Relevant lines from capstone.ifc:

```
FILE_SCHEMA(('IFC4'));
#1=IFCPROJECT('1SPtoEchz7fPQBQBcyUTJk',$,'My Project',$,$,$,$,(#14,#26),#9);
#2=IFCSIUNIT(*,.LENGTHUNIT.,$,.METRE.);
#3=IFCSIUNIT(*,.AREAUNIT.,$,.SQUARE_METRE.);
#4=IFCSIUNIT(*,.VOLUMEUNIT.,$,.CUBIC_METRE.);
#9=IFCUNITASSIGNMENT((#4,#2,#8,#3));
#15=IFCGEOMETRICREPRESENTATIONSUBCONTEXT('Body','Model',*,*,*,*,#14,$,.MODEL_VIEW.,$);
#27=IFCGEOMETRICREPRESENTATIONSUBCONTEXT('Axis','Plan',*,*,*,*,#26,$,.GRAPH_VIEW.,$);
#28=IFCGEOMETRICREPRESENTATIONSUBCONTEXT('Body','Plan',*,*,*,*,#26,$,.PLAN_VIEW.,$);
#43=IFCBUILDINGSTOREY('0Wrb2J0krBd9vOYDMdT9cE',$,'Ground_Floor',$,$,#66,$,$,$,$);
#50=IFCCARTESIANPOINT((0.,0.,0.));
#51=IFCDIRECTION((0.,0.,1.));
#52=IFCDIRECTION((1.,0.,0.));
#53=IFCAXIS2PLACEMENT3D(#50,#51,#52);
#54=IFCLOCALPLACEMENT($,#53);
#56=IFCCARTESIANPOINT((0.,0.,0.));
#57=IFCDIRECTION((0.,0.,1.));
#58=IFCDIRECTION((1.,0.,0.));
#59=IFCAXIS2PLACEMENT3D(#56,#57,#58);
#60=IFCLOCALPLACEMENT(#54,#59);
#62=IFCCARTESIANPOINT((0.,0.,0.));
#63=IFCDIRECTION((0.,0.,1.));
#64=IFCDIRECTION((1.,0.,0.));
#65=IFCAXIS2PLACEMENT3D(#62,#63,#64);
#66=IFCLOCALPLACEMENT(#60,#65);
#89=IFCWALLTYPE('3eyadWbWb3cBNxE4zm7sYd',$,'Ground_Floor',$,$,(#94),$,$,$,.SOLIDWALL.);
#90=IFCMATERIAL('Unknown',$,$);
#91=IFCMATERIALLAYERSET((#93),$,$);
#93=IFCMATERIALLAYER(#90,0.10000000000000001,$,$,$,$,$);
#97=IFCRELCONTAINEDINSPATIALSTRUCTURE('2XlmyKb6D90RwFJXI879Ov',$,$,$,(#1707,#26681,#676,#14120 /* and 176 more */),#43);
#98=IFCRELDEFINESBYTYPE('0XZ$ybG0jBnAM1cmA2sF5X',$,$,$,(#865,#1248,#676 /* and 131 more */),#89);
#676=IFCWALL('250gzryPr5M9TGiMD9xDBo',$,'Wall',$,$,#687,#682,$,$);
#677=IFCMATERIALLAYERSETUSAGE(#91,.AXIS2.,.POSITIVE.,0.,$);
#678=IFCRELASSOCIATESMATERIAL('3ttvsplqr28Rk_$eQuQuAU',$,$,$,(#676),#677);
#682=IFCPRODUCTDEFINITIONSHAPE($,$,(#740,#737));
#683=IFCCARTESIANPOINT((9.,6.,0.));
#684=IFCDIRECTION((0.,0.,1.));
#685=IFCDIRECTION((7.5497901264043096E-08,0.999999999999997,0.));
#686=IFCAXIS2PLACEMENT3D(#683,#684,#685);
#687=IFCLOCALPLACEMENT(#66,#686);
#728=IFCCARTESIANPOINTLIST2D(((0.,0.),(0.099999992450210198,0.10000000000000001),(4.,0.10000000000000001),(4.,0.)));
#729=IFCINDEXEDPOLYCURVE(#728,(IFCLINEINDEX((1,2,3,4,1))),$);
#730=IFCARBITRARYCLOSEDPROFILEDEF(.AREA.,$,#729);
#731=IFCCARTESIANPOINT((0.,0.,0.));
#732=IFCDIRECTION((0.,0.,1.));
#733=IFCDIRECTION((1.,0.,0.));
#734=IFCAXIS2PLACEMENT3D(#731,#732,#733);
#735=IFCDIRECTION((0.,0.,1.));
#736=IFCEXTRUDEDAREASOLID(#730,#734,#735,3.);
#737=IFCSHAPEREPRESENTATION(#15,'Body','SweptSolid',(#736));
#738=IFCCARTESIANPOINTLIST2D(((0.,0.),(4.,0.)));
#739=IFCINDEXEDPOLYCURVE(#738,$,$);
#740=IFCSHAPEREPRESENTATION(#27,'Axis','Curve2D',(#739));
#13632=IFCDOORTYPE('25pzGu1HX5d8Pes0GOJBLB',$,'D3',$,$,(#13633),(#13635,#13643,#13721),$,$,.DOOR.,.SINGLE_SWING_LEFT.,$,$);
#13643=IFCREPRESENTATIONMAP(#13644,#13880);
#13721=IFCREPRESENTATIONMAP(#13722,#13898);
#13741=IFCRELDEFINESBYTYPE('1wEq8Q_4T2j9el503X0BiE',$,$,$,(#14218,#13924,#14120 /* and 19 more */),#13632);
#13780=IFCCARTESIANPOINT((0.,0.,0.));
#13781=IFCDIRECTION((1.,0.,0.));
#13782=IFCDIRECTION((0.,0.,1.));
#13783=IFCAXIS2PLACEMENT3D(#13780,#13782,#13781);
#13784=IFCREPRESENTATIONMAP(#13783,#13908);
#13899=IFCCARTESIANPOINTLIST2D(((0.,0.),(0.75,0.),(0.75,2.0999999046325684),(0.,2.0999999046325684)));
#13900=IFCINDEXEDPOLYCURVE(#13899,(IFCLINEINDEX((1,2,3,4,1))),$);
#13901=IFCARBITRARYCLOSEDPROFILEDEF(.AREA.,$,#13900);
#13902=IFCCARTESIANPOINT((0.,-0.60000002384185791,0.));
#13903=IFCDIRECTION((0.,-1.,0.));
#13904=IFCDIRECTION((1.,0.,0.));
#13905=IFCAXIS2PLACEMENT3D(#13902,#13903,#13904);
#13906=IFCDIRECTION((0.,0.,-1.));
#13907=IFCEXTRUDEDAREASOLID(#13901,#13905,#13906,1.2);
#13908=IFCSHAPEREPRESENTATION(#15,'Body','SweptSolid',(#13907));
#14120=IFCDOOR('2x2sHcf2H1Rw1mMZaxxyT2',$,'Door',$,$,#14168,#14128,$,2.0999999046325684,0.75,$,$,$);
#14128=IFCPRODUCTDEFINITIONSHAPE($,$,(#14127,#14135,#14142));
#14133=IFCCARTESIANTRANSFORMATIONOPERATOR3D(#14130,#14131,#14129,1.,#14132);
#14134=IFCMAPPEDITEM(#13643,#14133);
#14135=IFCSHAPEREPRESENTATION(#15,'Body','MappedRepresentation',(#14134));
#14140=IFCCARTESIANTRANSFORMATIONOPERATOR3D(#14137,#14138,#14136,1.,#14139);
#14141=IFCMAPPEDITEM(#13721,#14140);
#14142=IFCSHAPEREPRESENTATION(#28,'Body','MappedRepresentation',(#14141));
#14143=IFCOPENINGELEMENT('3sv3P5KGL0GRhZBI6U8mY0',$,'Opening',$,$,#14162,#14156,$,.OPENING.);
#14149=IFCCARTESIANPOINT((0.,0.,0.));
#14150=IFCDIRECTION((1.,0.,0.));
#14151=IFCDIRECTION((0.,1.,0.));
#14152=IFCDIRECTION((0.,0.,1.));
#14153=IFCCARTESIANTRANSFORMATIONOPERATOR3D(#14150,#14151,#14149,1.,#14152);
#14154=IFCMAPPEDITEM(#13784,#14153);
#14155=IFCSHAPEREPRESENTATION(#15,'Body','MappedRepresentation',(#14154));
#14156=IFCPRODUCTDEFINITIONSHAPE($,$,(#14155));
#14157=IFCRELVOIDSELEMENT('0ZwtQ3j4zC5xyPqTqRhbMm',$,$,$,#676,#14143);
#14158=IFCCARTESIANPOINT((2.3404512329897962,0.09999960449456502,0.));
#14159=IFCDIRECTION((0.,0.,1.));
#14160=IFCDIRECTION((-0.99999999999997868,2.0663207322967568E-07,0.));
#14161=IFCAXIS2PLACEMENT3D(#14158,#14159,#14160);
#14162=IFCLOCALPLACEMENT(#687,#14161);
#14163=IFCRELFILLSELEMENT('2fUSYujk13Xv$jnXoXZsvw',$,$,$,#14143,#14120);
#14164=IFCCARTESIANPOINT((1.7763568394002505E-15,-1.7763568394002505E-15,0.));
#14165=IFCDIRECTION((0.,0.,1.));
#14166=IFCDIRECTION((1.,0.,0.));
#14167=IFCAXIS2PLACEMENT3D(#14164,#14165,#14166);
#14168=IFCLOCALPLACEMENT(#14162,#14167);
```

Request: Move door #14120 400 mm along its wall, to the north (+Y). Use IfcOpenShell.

```python
import ifcopenshell
import ifcopenshell.api.geometry
import ifcopenshell.util.placement
import ifcopenshell.util.unit

model = ifcopenshell.open("capstone.ifc")
unit_scale = ifcopenshell.util.unit.calculate_unit_scale(model)

door = model.by_guid("2x2sHcf2H1Rw1mMZaxxyT2")
opening = door.FillsVoids[0].RelatingOpeningElement
wall = opening.VoidsElements[0].RelatingBuildingElement

wall_matrix = ifcopenshell.util.placement.get_local_placement(wall.ObjectPlacement)
shift = wall_matrix[:3, 0] * 0.4 / unit_scale
before = ifcopenshell.util.placement.get_local_placement(door.ObjectPlacement)[:3, 3].copy()

# The door is placed relative to its opening, so it follows when the opening moves.
matrix = ifcopenshell.util.placement.get_local_placement(opening.ObjectPlacement)
matrix[:3, 3] += shift
ifcopenshell.api.geometry.edit_object_placement(
    model, product=opening, matrix=matrix, is_si=False, should_transform_children=True
)

after = ifcopenshell.util.placement.get_local_placement(door.ObjectPlacement)[:3, 3]
print("door moved by", (after - before).round(3) + 0.0)

model.write("capstone_edited.ifc")
```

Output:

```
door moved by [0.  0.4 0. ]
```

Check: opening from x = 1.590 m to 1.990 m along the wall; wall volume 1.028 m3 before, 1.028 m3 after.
